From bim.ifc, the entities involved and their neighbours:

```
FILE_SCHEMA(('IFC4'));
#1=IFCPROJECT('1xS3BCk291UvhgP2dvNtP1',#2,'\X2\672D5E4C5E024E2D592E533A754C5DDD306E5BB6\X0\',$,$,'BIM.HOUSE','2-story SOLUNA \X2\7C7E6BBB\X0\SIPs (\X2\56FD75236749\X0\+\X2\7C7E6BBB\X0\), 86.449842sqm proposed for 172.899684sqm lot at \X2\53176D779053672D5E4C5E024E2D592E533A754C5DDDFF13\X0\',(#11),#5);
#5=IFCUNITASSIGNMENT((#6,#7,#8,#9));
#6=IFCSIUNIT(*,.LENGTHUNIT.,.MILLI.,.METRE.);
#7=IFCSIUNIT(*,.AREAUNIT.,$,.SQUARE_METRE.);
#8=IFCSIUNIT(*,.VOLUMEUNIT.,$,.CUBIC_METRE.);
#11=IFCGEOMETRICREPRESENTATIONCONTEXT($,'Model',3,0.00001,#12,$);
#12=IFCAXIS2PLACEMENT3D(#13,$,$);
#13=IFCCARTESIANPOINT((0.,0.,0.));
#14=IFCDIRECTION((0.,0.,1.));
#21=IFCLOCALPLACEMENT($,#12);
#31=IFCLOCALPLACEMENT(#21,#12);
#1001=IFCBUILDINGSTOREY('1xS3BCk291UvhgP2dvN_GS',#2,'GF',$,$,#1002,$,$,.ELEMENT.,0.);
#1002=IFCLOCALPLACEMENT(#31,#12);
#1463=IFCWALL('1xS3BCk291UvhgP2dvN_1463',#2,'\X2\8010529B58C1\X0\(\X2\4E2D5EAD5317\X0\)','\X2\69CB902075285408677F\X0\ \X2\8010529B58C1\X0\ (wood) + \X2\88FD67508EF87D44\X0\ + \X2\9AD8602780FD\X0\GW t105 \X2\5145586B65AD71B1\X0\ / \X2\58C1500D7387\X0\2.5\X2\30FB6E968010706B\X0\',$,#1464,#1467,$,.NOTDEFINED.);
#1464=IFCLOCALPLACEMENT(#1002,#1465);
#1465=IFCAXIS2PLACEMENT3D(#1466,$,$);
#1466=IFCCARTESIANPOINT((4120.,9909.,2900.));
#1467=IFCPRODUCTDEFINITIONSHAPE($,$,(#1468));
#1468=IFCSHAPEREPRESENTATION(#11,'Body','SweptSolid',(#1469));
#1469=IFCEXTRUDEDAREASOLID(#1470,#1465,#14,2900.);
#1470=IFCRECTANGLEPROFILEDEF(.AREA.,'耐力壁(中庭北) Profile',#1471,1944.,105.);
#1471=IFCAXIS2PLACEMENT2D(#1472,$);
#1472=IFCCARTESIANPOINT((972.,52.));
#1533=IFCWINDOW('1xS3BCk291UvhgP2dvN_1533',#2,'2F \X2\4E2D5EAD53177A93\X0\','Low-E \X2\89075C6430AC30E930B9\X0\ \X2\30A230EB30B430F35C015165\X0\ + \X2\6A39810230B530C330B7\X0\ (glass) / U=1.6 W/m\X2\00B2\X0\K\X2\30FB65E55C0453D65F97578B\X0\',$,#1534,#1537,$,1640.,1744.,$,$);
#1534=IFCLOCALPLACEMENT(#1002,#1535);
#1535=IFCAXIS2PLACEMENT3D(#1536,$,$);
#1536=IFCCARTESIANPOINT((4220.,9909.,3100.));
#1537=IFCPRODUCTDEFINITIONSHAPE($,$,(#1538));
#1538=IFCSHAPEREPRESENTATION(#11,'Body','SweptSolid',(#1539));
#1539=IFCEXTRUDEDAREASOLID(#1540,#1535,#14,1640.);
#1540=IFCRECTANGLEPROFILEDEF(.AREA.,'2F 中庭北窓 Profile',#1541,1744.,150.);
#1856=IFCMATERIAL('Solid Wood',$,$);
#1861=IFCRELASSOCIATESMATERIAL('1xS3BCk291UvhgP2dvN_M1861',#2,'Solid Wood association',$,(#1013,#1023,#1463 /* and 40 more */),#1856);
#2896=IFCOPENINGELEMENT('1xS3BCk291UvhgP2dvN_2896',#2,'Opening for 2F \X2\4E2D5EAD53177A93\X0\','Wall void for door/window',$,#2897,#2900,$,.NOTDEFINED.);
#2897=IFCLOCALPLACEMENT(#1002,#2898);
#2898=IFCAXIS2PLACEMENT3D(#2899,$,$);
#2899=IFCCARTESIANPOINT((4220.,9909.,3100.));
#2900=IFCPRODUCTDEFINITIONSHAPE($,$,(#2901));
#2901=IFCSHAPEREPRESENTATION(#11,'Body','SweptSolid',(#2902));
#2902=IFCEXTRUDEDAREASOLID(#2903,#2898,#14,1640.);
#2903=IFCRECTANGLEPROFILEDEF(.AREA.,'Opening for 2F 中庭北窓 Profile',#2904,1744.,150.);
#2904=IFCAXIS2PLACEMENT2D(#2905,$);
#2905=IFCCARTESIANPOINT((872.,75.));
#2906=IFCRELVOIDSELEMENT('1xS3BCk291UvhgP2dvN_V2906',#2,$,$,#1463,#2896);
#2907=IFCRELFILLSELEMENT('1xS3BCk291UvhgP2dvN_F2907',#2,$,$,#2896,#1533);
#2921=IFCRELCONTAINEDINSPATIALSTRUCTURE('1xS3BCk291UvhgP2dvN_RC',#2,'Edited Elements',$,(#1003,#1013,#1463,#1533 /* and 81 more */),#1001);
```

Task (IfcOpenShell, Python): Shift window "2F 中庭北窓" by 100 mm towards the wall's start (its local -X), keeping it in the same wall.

```python
import ifcopenshell
import ifcopenshell.api.geometry
import ifcopenshell.util.placement

model = ifcopenshell.open("bim.ifc")

window = model.by_id(1533)
opening = window.FillsVoids[0].RelatingOpeningElement
wall = opening.VoidsElements[0].RelatingBuildingElement

wall_matrix = ifcopenshell.util.placement.get_local_placement(wall.ObjectPlacement)
shift = wall_matrix[:3, 0] * -100.0
before = ifcopenshell.util.placement.get_local_placement(window.ObjectPlacement)[:3, 3].copy()

# The window is not placed relative to its opening, so move both.
for product in (opening, window):
    matrix = ifcopenshell.util.placement.get_local_placement(product.ObjectPlacement)
    matrix[:3, 3] += shift
    ifcopenshell.api.geometry.edit_object_placement(model, product=product, matrix=matrix, is_si=False)

after = ifcopenshell.util.placement.get_local_placement(window.ObjectPlacement)[:3, 3]
print("window moved by", (after - before).round(3) + 0.0)

model.write("bim_rev.ifc")
```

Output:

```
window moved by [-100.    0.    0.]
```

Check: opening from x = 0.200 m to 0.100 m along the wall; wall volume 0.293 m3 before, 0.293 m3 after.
